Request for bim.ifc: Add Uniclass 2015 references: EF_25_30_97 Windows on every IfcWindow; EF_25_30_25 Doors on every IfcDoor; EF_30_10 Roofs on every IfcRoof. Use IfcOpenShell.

First a look at what the model holds.

```python
import ifcopenshell

model = ifcopenshell.open("bim.ifc")
print(model.schema)
print("classifications:", [c.Name for c in model.by_type("IfcClassification")])
for ifc_class in ("IfcDoor", "IfcRoof", "IfcStair", "IfcWall", "IfcWindow"):
    print(ifc_class, len(model.by_type(ifc_class)))
```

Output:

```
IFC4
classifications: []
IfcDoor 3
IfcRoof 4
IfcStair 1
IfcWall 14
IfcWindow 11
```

```python
import ifcopenshell
import ifcopenshell.api.classification

model = ifcopenshell.open("bim.ifc")

system = ifcopenshell.api.classification.add_classification(model, classification="Uniclass 2015")

codes = {
    "IfcWindow": ("EF_25_30_97", "Windows"),
    "IfcDoor": ("EF_25_30_25", "Doors"),
    "IfcRoof": ("EF_30_10", "Roofs"),
}
for ifc_class, (code, name) in codes.items():
    products = model.by_type(ifc_class)
    ifcopenshell.api.classification.add_reference(
        model, products=products, classification=system, identification=code, name=name
    )
    print(code, len(products))

model.write("bim-out.ifc")
```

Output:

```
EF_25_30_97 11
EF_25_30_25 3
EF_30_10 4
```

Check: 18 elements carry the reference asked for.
